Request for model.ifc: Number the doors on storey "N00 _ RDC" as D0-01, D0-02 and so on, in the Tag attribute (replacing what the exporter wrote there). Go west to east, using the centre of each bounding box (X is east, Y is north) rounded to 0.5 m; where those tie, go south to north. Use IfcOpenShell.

First a look at what the model holds.

```python
import ifcopenshell
import ifcopenshell.util.element
import ifcopenshell.util.placement

model = ifcopenshell.open("model.ifc")
print(model.schema)
storey = next(s for s in model.by_type("IfcBuildingStorey") if s.Name == "N00 _ RDC")
doors = [e for e in ifcopenshell.util.element.get_decomposition(storey) if e.is_a("IfcDoor")]
for e in sorted(doors, key=lambda e: e.id()):
    origin = ifcopenshell.util.placement.get_local_placement(e.ObjectPlacement)[:3, 3]
    print(e.id(), e.Tag, e.Name, origin.round(2) + 0.0, sep=" | ")
```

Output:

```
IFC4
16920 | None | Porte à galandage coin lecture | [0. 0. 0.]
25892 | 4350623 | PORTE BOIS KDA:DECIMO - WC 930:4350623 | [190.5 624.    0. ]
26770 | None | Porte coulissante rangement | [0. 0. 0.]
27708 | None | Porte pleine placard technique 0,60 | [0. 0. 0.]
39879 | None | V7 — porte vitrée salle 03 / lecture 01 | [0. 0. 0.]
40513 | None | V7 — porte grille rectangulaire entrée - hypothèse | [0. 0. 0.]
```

```python
import ifcopenshell
import ifcopenshell.geom
import ifcopenshell.util.element
import ifcopenshell.util.shape

model = ifcopenshell.open("model.ifc")
settings = ifcopenshell.geom.settings()
settings.set("use-world-coords", True)


def centre(element):
    shape = ifcopenshell.geom.create_shape(settings, element)
    return ifcopenshell.util.shape.get_bbox_centroid(shape.geometry)


storey = next(s for s in model.by_type("IfcBuildingStorey") if s.Name == "N00 _ RDC")
doors = [e for e in ifcopenshell.util.element.get_decomposition(storey) if e.is_a("IfcDoor")]

# Insertion points can sit at a corner or the storey origin, so sort by the geometry (in metres).
centres = {e: centre(e) for e in doors}
doors.sort(key=lambda e: (round(centres[e][0] / 0.5), centres[e][1]))

for i, e in enumerate(doors, start=1):
    number = f"D0-{i:02d}"
    e.Tag = number
    print(e.id(), number)

model.write("model_updated.ifc")
```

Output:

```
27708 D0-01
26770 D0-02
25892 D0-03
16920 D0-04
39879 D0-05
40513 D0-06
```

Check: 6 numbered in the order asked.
